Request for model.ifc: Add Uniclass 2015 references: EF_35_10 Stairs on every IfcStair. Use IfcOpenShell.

First a look at what the model holds.

```python
import ifcopenshell

model = ifcopenshell.open("model.ifc")
print(model.schema)
print("classifications:", [c.Name for c in model.by_type("IfcClassification")])
for ifc_class in ("IfcDoor", "IfcRoof", "IfcStair", "IfcWall", "IfcWindow"):
    print(ifc_class, len(model.by_type(ifc_class)))
```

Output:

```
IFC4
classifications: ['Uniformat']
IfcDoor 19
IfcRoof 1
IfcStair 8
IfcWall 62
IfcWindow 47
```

```python
import ifcopenshell
import ifcopenshell.api.classification

model = ifcopenshell.open("model.ifc")

system = ifcopenshell.api.classification.add_classification(model, classification="Uniclass 2015")

codes = {
    "IfcStair": ("EF_35_10", "Stairs"),
}
for ifc_class, (code, name) in codes.items():
    products = model.by_type(ifc_class)
    ifcopenshell.api.classification.add_reference(
        model, products=products, classification=system, identification=code, name=name
    )
    print(code, len(products))

model.write("model-out.ifc")
```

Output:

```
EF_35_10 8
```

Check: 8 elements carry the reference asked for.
